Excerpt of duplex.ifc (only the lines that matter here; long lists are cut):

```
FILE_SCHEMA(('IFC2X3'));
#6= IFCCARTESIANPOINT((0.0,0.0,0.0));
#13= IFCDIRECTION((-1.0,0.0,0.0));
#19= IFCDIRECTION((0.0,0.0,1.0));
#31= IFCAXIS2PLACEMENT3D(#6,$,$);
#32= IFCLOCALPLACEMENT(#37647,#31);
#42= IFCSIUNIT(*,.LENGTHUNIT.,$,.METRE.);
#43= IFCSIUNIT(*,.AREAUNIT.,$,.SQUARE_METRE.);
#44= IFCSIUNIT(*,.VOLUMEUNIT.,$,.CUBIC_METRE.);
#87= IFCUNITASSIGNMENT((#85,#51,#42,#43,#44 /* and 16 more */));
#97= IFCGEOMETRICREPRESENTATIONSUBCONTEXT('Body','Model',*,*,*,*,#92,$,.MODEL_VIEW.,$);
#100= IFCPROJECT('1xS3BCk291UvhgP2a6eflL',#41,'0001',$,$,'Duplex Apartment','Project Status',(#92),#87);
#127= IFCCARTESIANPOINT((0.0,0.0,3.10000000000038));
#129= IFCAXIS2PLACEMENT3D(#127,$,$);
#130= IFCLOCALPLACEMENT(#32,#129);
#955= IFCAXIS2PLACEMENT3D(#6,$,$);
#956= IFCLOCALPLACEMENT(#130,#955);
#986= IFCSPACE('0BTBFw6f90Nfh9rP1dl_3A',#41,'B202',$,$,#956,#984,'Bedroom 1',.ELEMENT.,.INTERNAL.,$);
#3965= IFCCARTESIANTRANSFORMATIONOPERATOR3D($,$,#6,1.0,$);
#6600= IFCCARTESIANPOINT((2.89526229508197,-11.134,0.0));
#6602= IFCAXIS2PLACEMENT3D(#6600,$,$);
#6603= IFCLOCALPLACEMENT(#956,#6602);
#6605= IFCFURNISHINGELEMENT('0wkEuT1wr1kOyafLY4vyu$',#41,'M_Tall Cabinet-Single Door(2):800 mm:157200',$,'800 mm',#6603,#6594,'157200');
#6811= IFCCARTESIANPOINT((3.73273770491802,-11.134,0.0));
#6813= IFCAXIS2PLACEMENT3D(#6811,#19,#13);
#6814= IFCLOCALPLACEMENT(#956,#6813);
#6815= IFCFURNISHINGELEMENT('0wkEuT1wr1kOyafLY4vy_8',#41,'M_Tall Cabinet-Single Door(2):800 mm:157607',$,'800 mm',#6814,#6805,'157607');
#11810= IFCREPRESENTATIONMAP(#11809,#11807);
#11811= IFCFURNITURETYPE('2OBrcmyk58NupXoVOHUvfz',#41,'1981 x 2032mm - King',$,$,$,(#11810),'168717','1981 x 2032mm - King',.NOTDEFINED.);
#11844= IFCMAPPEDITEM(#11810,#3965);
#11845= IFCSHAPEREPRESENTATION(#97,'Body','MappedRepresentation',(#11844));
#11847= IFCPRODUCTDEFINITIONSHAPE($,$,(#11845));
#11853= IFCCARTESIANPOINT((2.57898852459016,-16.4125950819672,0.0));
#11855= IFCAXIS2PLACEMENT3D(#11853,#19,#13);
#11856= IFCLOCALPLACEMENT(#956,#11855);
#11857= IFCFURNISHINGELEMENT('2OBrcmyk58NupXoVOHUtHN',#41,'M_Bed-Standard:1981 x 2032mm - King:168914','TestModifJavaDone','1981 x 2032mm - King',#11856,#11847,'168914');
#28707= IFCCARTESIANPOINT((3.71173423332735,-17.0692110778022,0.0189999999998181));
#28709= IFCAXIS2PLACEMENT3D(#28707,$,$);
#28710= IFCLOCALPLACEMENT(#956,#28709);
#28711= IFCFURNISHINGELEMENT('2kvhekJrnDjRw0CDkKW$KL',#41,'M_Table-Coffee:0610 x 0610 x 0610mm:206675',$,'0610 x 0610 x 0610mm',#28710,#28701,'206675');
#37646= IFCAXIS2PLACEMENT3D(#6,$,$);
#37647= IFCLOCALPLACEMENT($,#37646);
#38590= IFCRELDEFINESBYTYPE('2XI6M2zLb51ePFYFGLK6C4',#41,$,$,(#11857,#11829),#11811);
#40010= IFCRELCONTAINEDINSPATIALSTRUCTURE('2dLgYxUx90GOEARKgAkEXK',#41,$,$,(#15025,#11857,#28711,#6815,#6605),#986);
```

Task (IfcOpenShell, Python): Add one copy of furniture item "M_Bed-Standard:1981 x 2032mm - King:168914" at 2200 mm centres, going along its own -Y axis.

```python
import ifcopenshell
import ifcopenshell.api.geometry
import ifcopenshell.api.root
import ifcopenshell.util.element
import ifcopenshell.util.placement
import ifcopenshell.util.unit

model = ifcopenshell.open("duplex.ifc")
unit_scale = ifcopenshell.util.unit.calculate_unit_scale(model)


def reuse_history(source, copy):
    """copy_class also copies each property set's owner history, people and application; keep the originals."""
    for rel in copy.IsDefinedBy:
        if rel.is_a("IfcRelDefinesByProperties") and (history := rel.RelatingPropertyDefinition.OwnerHistory):
            rel.RelatingPropertyDefinition.OwnerHistory = source.OwnerHistory
            ifcopenshell.util.element.remove_deep2(model, history)


source = model.by_guid("2OBrcmyk58NupXoVOHUtHN")
base = ifcopenshell.util.placement.get_local_placement(source.ObjectPlacement)
step = -base[:3, 1] * 2.2 / unit_scale

for i in range(1, 2):
    copy = ifcopenshell.api.root.copy_class(model, product=source)
    copy.Representation = ifcopenshell.util.element.copy_deep(
        model, source.Representation, exclude=["IfcGeometricRepresentationContext", "IfcRepresentationMap"]
    )
    copy.Name = "M_Bed-Standard:1981 x 2032mm - King"
    copy.Tag = None
    reuse_history(source, copy)
    matrix = base.copy()
    matrix[:3, 3] += i * step
    print("added at", matrix[:3, 3].round(3) + 0.0)
    ifcopenshell.api.geometry.edit_object_placement(model, product=copy, matrix=matrix, is_si=False)

model.write("duplex_v2.ifc")
```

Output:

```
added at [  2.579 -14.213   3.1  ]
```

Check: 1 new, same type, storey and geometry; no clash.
